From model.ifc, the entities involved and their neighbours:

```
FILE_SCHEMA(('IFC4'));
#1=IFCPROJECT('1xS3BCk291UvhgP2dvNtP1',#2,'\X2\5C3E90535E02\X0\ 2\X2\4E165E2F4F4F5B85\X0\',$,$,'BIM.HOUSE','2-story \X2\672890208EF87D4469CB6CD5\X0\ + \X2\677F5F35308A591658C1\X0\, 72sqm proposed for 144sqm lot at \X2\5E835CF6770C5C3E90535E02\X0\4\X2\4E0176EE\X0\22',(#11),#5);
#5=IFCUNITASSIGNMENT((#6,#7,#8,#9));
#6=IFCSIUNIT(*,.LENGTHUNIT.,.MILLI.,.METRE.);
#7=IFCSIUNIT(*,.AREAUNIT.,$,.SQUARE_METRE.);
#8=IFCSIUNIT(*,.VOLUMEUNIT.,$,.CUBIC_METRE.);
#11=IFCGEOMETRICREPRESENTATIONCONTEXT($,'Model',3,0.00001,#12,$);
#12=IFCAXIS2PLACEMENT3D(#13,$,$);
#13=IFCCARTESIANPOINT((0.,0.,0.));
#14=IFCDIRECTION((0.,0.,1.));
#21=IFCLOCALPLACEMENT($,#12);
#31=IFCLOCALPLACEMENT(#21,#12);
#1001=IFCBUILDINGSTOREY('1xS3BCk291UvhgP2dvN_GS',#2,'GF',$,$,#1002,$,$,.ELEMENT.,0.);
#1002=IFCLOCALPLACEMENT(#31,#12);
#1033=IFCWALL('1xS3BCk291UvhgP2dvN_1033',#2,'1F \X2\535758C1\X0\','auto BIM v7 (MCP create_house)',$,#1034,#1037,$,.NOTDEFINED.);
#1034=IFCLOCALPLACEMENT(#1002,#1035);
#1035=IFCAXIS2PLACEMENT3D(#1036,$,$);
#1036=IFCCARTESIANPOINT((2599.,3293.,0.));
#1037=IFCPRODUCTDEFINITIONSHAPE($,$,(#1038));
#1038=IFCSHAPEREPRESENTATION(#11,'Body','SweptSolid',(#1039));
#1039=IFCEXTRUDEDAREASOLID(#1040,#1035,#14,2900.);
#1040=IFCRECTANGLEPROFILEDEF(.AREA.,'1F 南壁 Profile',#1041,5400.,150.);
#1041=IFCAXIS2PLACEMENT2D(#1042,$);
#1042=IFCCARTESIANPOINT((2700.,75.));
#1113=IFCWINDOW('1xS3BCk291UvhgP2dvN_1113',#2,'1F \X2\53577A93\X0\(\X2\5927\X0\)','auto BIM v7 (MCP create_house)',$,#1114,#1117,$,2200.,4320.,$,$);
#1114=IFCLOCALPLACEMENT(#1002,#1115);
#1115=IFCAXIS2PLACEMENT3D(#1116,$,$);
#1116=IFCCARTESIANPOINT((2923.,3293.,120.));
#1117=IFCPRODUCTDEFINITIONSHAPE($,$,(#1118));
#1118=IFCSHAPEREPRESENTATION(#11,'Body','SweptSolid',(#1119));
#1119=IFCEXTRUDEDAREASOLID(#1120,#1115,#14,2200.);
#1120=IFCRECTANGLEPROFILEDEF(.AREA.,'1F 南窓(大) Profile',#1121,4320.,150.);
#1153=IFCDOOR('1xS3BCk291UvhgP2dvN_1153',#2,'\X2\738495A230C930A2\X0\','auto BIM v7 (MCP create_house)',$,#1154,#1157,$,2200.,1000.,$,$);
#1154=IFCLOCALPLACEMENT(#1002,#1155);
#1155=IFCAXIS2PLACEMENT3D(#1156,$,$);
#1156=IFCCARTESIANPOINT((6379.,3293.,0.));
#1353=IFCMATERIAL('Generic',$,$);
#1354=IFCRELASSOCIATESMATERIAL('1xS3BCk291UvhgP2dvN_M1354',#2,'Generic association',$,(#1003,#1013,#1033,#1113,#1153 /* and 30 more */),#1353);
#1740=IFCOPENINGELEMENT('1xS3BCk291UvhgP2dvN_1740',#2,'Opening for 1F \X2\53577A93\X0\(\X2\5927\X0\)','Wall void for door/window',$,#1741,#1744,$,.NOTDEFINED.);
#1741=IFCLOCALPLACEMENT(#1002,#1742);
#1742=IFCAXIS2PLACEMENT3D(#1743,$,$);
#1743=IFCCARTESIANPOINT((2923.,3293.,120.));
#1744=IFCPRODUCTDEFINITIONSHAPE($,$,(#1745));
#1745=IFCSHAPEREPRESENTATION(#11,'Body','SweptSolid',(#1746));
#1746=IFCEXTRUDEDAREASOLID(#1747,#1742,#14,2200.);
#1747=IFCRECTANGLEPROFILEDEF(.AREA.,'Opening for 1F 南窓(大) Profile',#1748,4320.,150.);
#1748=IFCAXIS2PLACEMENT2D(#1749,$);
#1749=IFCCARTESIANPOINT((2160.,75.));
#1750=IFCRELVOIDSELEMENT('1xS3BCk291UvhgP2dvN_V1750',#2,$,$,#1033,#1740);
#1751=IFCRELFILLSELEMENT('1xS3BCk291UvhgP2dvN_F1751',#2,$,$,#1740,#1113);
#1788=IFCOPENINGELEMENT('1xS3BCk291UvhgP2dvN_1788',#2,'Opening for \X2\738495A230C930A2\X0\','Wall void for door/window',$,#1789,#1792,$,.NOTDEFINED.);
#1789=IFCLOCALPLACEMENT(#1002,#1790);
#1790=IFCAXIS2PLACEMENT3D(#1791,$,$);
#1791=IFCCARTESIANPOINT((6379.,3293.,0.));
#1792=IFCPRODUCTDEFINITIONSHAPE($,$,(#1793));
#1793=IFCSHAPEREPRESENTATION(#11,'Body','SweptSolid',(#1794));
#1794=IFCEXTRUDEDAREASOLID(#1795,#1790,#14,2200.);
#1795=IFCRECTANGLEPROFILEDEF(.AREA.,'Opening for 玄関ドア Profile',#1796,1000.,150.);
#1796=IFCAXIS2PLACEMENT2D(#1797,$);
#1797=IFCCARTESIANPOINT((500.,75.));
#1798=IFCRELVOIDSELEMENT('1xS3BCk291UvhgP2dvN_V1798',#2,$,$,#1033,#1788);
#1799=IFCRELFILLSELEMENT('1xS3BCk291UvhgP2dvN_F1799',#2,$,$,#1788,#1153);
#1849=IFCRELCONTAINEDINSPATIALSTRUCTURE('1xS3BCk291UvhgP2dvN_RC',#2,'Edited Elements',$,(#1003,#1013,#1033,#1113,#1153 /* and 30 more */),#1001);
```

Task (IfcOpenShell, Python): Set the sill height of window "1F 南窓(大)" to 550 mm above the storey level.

```python
import numpy as np
import ifcopenshell
import ifcopenshell.api.geometry
import ifcopenshell.geom
import ifcopenshell.util.element
import ifcopenshell.util.placement
import ifcopenshell.util.shape
import ifcopenshell.util.unit

model = ifcopenshell.open("model.ifc")
unit_scale = ifcopenshell.util.unit.calculate_unit_scale(model)

window = model.by_guid("1xS3BCk291UvhgP2dvN_1113")
opening = window.FillsVoids[0].RelatingOpeningElement
storey = ifcopenshell.util.element.get_container(window, ifc_class="IfcBuildingStorey")
level = ifcopenshell.util.placement.get_local_placement(storey.ObjectPlacement)[2, 3]

# The opening's origin need not be at the sill, so measure its lowest point.
shape = ifcopenshell.geom.create_shape(ifcopenshell.geom.settings(), opening)
bottom = ifcopenshell.util.shape.get_shape_bottom_elevation(shape, shape.geometry) / unit_scale
dz = level + 550.0 - bottom

shift = np.array([0.0, 0.0, dz])
# The window is not placed relative to its opening, so move both.
for product in (opening, window):
    matrix = ifcopenshell.util.placement.get_local_placement(product.ObjectPlacement)
    matrix[:3, 3] += shift
    ifcopenshell.api.geometry.edit_object_placement(model, product=product, matrix=matrix, is_si=False)

print(f"moved by {dz * unit_scale:+.3f} m")

model.write("model-out.ifc")
```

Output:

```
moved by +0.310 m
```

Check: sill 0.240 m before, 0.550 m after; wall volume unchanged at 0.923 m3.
